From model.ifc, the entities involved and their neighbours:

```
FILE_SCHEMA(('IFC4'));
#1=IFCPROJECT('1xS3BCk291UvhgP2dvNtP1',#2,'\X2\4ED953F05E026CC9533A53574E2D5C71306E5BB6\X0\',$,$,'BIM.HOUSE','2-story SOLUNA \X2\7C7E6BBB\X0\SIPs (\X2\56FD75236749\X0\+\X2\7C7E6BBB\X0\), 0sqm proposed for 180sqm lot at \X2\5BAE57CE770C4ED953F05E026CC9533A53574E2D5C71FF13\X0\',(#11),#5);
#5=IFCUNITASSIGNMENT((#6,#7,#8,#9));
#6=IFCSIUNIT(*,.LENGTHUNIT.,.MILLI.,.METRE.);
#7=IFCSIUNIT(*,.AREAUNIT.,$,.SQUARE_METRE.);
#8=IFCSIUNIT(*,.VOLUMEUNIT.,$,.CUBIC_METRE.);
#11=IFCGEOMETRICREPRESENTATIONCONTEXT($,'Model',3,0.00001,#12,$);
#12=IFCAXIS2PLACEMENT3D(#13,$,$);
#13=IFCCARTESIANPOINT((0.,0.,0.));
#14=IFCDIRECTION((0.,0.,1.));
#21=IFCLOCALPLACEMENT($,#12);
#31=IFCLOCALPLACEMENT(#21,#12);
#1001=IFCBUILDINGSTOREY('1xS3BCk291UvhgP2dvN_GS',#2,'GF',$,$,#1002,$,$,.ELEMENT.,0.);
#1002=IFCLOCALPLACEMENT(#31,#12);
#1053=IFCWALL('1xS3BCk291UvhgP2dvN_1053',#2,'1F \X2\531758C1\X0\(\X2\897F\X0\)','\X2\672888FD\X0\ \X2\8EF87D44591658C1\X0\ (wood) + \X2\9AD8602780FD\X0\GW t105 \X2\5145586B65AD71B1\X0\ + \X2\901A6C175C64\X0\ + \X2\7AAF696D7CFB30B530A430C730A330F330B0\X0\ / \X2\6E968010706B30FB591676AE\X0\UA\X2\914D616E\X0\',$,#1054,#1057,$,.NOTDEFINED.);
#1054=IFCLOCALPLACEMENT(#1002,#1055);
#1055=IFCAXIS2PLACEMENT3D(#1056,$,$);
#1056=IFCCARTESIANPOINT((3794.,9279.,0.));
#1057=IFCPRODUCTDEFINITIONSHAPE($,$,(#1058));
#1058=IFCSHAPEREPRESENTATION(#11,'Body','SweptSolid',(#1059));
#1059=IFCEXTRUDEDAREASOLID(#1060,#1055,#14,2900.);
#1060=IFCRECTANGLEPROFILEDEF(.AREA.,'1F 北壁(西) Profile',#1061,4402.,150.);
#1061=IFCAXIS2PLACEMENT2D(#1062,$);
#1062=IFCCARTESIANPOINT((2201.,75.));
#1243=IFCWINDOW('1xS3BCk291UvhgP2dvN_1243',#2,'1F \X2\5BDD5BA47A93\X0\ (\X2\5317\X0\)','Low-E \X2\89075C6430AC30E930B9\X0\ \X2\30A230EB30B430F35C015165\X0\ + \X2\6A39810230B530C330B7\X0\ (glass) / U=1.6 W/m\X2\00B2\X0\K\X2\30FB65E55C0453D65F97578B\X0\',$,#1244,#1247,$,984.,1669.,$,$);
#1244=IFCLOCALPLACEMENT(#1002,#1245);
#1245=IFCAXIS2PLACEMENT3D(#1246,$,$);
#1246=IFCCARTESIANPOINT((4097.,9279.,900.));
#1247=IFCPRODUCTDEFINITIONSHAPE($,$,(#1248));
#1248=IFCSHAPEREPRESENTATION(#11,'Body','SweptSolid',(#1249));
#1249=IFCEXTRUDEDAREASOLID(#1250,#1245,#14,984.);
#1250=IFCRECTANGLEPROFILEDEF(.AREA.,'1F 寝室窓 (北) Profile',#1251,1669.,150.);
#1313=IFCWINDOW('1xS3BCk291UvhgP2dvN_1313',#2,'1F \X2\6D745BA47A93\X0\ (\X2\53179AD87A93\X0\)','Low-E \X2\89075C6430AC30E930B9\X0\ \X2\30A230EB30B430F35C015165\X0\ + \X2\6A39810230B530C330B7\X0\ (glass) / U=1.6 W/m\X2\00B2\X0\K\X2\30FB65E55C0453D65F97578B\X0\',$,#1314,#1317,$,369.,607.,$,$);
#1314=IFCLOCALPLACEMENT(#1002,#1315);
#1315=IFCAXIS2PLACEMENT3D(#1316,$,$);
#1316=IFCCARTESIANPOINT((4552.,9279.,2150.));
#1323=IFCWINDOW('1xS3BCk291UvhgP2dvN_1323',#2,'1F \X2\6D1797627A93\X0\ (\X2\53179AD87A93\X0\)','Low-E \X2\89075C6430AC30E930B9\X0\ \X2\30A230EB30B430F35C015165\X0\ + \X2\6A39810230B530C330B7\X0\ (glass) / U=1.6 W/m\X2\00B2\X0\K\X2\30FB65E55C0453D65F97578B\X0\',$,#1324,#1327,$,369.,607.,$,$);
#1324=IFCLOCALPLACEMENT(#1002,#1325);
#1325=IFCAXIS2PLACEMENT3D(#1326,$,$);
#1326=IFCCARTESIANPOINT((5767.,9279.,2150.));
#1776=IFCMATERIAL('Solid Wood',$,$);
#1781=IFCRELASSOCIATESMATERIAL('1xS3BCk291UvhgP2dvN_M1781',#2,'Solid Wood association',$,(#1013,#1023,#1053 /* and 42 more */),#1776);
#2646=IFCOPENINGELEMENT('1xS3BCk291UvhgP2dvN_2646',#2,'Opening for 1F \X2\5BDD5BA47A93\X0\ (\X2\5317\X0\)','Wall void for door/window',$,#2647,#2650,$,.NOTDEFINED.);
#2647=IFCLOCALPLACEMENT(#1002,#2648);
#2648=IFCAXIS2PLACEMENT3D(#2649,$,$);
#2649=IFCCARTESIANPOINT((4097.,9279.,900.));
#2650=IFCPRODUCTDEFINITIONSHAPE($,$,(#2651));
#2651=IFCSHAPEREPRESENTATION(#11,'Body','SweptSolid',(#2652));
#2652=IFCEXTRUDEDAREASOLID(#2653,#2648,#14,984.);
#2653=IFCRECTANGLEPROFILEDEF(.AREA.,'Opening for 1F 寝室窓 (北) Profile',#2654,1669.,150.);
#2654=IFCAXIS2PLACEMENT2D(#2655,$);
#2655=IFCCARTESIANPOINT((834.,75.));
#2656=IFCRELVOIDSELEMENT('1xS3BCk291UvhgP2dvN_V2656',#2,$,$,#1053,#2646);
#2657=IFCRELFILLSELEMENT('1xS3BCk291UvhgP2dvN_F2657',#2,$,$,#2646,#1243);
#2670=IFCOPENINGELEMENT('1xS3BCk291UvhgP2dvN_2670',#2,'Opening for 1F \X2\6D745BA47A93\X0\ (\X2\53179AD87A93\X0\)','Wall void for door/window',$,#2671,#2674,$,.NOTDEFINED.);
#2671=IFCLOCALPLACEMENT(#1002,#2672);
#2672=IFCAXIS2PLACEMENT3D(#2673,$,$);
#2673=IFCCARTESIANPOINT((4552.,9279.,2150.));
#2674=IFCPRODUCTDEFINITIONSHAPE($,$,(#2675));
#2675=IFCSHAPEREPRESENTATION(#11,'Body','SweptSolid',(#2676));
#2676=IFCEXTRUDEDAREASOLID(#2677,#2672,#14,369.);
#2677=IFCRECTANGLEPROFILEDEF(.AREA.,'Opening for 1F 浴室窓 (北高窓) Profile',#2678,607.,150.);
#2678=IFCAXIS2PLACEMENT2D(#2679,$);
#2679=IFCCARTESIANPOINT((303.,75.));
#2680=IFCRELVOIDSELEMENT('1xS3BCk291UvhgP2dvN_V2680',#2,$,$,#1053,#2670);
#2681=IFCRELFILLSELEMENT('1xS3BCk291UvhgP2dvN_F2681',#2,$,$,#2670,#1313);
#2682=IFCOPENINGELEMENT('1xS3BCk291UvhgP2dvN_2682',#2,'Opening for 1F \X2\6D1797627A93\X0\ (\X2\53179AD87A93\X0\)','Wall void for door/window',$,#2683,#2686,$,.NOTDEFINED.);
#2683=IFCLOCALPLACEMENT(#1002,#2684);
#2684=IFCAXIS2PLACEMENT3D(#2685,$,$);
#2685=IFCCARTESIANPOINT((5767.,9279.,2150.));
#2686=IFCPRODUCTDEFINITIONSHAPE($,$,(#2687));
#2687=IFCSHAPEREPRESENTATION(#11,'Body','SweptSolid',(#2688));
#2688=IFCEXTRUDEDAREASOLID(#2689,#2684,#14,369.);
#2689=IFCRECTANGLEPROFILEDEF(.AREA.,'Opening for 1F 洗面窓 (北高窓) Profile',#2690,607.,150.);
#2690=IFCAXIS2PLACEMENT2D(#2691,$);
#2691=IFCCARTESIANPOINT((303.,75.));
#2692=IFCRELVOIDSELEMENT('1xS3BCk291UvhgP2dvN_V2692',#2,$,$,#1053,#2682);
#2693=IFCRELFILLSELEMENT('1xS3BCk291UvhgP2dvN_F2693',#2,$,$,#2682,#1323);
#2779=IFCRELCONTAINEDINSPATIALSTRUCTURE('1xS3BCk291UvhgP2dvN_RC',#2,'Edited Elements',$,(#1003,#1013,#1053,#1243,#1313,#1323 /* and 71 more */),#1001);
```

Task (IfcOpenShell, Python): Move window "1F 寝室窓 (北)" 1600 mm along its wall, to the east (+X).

```python
import ifcopenshell
import ifcopenshell.api.geometry
import ifcopenshell.util.placement
import ifcopenshell.util.unit

model = ifcopenshell.open("model.ifc")
unit_scale = ifcopenshell.util.unit.calculate_unit_scale(model)

window = model.by_guid("1xS3BCk291UvhgP2dvN_1243")
opening = window.FillsVoids[0].RelatingOpeningElement
wall = opening.VoidsElements[0].RelatingBuildingElement

wall_matrix = ifcopenshell.util.placement.get_local_placement(wall.ObjectPlacement)
shift = wall_matrix[:3, 0] * 1.6 / unit_scale
before = ifcopenshell.util.placement.get_local_placement(window.ObjectPlacement)[:3, 3].copy()

# The window is not placed relative to its opening, so move both.
for product in (opening, window):
    matrix = ifcopenshell.util.placement.get_local_placement(product.ObjectPlacement)
    matrix[:3, 3] += shift
    ifcopenshell.api.geometry.edit_object_placement(model, product=product, matrix=matrix, is_si=False)

after = ifcopenshell.util.placement.get_local_placement(window.ObjectPlacement)[:3, 3]
print("window moved by", (after - before).round(3) + 0.0)

model.write("model_v2.ifc")
```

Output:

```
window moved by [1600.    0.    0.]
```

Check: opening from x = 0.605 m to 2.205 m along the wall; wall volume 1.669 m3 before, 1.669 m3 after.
